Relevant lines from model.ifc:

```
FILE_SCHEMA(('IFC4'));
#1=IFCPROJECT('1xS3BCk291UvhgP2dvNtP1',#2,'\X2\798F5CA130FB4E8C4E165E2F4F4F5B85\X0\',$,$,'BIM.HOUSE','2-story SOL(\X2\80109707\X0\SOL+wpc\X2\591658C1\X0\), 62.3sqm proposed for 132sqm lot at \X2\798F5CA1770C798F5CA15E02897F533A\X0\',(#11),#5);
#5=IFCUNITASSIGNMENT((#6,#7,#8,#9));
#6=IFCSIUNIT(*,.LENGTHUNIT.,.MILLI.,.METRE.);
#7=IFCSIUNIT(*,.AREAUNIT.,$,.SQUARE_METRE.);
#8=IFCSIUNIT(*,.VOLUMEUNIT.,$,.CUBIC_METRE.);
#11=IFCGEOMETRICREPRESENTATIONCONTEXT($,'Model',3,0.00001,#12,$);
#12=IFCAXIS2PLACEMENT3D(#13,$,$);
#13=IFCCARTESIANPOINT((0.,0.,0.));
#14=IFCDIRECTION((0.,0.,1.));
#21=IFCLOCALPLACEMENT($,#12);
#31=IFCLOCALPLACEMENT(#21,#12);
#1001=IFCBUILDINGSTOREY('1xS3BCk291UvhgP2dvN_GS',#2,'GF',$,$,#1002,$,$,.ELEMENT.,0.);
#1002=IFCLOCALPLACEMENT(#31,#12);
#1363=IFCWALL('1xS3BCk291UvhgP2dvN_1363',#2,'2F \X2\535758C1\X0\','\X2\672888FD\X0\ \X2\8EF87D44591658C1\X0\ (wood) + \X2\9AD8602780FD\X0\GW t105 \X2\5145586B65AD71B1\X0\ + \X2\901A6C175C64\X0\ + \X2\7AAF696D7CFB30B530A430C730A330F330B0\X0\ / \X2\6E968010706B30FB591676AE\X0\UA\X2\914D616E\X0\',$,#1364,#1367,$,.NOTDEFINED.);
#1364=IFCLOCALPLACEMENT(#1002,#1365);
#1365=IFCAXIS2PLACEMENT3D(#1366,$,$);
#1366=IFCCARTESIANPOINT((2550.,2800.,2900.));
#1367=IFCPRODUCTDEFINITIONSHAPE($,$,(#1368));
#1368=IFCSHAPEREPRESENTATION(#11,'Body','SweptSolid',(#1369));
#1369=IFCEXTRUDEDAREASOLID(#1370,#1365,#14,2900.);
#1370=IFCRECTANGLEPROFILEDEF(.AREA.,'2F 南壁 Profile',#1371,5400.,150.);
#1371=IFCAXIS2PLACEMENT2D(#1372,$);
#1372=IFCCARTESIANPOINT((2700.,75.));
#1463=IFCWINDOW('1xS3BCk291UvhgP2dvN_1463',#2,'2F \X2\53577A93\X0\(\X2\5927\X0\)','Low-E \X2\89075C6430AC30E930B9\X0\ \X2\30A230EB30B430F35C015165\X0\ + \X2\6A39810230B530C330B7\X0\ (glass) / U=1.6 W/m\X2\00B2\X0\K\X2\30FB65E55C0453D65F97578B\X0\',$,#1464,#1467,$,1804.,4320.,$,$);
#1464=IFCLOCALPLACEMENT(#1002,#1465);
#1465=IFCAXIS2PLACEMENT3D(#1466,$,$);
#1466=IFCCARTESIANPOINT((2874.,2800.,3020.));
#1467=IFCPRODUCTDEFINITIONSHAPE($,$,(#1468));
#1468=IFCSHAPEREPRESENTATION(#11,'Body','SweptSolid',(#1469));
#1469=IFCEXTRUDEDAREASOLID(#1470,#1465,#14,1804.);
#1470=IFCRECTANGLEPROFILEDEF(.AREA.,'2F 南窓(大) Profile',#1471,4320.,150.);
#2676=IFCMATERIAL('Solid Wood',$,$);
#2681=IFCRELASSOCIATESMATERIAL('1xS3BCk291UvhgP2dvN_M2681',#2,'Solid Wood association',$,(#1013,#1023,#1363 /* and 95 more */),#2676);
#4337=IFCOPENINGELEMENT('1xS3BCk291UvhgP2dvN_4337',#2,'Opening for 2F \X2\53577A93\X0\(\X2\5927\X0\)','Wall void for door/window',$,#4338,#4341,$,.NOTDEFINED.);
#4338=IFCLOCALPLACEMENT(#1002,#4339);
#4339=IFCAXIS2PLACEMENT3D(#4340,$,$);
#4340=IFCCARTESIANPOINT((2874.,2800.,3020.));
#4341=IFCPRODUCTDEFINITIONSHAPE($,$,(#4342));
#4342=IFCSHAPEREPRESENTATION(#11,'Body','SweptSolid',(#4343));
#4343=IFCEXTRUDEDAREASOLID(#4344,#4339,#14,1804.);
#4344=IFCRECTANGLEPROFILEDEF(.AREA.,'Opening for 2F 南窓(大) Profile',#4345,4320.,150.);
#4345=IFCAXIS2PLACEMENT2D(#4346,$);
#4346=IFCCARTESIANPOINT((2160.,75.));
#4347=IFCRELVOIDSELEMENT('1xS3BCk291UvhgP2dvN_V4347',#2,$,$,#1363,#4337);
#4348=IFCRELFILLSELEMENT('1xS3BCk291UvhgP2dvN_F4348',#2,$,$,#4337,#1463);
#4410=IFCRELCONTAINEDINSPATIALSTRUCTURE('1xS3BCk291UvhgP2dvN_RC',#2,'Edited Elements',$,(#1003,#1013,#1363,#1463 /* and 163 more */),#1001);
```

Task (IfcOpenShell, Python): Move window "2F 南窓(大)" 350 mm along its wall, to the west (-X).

```python
import ifcopenshell
import ifcopenshell.api.geometry
import ifcopenshell.util.placement
import ifcopenshell.util.unit

model = ifcopenshell.open("model.ifc")
unit_scale = ifcopenshell.util.unit.calculate_unit_scale(model)

window = model.by_guid("1xS3BCk291UvhgP2dvN_1463")
opening = window.FillsVoids[0].RelatingOpeningElement
wall = opening.VoidsElements[0].RelatingBuildingElement

wall_matrix = ifcopenshell.util.placement.get_local_placement(wall.ObjectPlacement)
shift = wall_matrix[:3, 0] * -0.35 / unit_scale
before = ifcopenshell.util.placement.get_local_placement(window.ObjectPlacement)[:3, 3].copy()

# The window is not placed relative to its opening, so move both.
for product in (opening, window):
    matrix = ifcopenshell.util.placement.get_local_placement(product.ObjectPlacement)
    matrix[:3, 3] += shift
    ifcopenshell.api.geometry.edit_object_placement(model, product=product, matrix=matrix, is_si=False)

after = ifcopenshell.util.placement.get_local_placement(window.ObjectPlacement)[:3, 3]
print("window moved by", (after - before).round(3) + 0.0)

model.write("model_v2.ifc")
```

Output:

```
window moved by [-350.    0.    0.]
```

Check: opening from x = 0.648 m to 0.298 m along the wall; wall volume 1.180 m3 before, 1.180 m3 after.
